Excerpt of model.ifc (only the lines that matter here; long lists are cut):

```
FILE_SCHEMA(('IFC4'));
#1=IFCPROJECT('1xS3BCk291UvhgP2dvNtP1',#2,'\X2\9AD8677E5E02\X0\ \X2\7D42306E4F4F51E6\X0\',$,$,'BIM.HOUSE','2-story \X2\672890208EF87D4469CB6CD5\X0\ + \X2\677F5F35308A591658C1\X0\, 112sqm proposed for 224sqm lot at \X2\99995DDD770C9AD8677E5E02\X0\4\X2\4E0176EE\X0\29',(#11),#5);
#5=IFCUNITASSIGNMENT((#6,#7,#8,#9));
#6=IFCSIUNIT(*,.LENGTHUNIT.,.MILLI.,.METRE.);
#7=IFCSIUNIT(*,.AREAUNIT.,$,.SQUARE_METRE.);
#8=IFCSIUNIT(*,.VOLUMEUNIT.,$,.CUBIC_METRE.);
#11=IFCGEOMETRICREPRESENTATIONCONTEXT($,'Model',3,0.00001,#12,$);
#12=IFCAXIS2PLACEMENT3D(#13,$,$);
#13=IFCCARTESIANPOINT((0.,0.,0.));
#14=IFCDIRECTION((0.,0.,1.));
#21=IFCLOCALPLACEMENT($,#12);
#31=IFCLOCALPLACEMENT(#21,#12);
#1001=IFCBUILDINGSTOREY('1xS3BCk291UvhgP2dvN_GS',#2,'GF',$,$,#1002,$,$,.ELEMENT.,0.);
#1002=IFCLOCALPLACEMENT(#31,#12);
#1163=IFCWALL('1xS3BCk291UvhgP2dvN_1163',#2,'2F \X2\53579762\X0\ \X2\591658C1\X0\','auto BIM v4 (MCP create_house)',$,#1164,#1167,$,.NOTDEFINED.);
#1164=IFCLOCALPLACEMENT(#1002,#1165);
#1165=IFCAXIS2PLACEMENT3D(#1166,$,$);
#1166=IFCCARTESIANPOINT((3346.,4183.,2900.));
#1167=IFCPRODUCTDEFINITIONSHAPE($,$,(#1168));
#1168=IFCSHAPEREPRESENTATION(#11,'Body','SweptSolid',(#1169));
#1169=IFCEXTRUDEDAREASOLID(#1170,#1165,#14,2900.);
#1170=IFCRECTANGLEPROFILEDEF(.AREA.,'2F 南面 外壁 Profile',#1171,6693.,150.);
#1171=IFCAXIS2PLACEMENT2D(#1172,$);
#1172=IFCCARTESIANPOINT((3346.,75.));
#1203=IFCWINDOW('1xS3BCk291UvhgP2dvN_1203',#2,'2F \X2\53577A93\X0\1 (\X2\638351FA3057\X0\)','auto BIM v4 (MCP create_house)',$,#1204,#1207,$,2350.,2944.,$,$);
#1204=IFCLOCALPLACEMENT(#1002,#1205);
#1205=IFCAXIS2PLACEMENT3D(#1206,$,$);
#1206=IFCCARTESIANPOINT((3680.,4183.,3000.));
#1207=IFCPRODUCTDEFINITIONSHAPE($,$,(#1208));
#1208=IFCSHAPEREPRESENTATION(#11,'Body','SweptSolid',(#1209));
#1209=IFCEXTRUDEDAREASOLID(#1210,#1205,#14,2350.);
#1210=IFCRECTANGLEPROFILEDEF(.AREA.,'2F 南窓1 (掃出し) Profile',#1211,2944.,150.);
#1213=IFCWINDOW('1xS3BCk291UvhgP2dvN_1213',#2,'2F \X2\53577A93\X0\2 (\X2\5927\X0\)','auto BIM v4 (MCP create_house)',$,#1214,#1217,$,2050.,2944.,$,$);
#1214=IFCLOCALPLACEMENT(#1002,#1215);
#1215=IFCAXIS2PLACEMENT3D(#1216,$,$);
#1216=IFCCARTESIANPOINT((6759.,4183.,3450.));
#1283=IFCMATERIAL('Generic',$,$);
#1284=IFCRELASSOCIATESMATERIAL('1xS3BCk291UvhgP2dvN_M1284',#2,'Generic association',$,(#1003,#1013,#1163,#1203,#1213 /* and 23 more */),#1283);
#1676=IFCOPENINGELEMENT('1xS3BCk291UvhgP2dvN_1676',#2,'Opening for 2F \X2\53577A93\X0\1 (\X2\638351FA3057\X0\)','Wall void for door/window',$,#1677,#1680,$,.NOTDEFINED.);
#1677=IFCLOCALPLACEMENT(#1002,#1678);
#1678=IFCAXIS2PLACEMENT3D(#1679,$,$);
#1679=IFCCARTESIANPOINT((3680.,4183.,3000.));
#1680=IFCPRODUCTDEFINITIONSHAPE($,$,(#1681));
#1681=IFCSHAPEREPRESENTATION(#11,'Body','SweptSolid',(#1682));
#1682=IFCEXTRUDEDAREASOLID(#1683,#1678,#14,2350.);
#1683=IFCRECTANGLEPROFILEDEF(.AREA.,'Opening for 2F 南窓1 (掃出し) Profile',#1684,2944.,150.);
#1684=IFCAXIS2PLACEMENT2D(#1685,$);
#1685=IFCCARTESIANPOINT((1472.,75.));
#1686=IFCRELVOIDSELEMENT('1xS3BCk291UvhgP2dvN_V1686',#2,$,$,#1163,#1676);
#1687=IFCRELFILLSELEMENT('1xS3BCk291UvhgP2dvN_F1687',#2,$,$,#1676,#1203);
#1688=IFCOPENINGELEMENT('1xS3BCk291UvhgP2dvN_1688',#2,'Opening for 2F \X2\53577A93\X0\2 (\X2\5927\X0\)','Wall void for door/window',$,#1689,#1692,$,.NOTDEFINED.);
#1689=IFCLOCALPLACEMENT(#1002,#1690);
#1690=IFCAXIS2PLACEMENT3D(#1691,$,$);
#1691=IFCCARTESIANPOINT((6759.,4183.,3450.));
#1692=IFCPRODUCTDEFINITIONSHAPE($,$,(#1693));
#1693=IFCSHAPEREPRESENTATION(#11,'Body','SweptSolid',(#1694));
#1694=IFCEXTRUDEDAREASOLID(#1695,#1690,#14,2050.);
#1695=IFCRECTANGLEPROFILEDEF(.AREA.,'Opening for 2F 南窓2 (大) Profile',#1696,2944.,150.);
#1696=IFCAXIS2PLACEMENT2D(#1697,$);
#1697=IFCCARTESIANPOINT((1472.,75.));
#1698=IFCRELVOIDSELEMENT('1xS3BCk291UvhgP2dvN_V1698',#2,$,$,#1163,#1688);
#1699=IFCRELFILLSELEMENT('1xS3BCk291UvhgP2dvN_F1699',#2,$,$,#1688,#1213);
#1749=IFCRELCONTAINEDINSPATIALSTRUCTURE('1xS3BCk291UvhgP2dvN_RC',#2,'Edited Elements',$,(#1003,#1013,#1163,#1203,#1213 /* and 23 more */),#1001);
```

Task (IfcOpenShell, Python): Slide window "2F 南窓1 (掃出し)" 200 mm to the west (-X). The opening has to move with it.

```python
import ifcopenshell
import ifcopenshell.api.geometry
import ifcopenshell.util.placement
import ifcopenshell.util.unit

model = ifcopenshell.open("model.ifc")
unit_scale = ifcopenshell.util.unit.calculate_unit_scale(model)

window = model.by_id(1203)
opening = window.FillsVoids[0].RelatingOpeningElement
wall = opening.VoidsElements[0].RelatingBuildingElement

wall_matrix = ifcopenshell.util.placement.get_local_placement(wall.ObjectPlacement)
shift = wall_matrix[:3, 0] * -0.2 / unit_scale
before = ifcopenshell.util.placement.get_local_placement(window.ObjectPlacement)[:3, 3].copy()

# The window is not placed relative to its opening, so move both.
for product in (opening, window):
    matrix = ifcopenshell.util.placement.get_local_placement(product.ObjectPlacement)
    matrix[:3, 3] += shift
    ifcopenshell.api.geometry.edit_object_placement(model, product=product, matrix=matrix, is_si=False)

after = ifcopenshell.util.placement.get_local_placement(window.ObjectPlacement)[:3, 3]
print("window moved by", (after - before).round(3) + 0.0)

model.write("model_edited.ifc")
```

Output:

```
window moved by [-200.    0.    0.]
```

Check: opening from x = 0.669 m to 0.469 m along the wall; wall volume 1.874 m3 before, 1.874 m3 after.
